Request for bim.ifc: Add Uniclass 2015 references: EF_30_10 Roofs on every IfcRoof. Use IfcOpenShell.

First a look at what the model holds.

```python
import ifcopenshell

model = ifcopenshell.open("bim.ifc")
print(model.schema)
print("classifications:", [c.Name for c in model.by_type("IfcClassification")])
for ifc_class in ("IfcDoor", "IfcRoof", "IfcStair", "IfcWall", "IfcWindow"):
    print(ifc_class, len(model.by_type(ifc_class)))
```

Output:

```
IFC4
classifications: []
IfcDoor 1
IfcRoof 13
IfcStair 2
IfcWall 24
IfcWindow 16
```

```python
import ifcopenshell
import ifcopenshell.api.classification

model = ifcopenshell.open("bim.ifc")

system = ifcopenshell.api.classification.add_classification(model, classification="Uniclass 2015")

codes = {
    "IfcRoof": ("EF_30_10", "Roofs"),
}
for ifc_class, (code, name) in codes.items():
    products = model.by_type(ifc_class)
    ifcopenshell.api.classification.add_reference(
        model, products=products, classification=system, identification=code, name=name
    )
    print(code, len(products))

model.write("bim_edited.ifc")
```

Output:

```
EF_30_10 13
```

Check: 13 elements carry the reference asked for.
